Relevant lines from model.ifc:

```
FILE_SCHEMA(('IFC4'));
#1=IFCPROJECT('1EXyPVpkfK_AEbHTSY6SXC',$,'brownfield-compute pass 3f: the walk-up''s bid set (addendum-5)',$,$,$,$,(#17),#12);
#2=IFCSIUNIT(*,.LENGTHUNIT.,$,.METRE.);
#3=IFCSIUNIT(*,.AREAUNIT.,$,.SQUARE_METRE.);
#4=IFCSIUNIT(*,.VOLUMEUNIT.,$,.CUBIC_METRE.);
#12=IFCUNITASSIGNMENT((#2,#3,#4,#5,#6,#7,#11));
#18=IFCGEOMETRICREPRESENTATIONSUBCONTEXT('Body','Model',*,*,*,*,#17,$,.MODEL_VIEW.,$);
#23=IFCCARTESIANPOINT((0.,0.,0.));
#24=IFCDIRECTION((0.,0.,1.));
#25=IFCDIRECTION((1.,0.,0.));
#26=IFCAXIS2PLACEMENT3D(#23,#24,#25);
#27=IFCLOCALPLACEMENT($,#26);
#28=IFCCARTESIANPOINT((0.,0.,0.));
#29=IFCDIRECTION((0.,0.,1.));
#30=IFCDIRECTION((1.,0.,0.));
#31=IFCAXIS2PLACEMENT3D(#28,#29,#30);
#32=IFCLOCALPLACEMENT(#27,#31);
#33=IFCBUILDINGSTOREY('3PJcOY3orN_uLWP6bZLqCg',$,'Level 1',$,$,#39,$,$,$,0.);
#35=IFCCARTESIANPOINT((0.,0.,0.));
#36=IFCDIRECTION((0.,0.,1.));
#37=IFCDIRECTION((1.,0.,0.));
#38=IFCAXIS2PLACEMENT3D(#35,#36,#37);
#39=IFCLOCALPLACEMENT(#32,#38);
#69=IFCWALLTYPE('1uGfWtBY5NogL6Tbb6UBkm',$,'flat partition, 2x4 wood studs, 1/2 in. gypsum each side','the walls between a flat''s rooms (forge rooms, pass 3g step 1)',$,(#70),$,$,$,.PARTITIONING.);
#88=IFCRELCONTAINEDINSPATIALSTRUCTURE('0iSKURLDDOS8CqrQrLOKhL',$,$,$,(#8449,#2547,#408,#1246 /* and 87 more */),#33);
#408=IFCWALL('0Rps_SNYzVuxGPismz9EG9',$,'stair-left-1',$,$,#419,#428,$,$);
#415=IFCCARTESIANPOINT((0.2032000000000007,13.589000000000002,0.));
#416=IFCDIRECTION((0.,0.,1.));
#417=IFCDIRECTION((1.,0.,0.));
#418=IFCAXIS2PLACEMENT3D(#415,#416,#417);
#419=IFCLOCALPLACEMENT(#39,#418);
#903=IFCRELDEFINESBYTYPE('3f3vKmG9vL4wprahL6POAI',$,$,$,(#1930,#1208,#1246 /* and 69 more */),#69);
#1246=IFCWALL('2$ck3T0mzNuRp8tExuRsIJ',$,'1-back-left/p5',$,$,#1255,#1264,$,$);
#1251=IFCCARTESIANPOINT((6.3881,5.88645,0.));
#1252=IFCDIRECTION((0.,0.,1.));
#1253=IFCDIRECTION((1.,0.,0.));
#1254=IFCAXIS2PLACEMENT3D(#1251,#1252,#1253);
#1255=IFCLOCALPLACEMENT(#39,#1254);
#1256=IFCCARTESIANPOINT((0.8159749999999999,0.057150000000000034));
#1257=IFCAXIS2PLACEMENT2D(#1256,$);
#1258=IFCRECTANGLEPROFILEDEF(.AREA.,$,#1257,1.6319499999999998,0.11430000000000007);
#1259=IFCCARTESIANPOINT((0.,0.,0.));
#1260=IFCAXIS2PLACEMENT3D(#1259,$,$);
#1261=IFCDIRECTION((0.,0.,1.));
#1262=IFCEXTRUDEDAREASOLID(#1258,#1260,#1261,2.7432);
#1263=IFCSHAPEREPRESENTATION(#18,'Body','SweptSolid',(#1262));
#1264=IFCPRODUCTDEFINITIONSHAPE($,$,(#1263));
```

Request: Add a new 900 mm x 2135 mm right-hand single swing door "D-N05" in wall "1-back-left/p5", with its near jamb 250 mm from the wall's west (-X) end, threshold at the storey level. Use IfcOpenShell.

```python
import numpy as np
import ifcopenshell
import ifcopenshell.api.feature
import ifcopenshell.api.geometry
import ifcopenshell.api.root
import ifcopenshell.api.spatial
import ifcopenshell.geom
import ifcopenshell.util.element
import ifcopenshell.util.placement
import ifcopenshell.util.representation
import ifcopenshell.util.shape
import ifcopenshell.util.unit

model = ifcopenshell.open("model.ifc")
unit_scale = ifcopenshell.util.unit.calculate_unit_scale(model)
settings = ifcopenshell.geom.settings()


def volume(element):
    """Net volume in cubic metres, openings subtracted."""
    shape = ifcopenshell.geom.create_shape(settings, element)
    return ifcopenshell.util.shape.get_volume(shape.geometry)


wall = model.by_guid("2$ck3T0mzNuRp8tExuRsIJ")
storey = ifcopenshell.util.element.get_container(wall, ifc_class="IfcBuildingStorey")
context = ifcopenshell.util.representation.get_context(model, "Model", "Body", "MODEL_VIEW")
before = volume(wall)

width, height, from_end, sill = 0.9, 2.135, 0.25, 0.0  # metres

# The wall runs along its own X axis, and the end named is its -X end.
wall_shape = ifcopenshell.geom.create_shape(settings, wall)
x, y, z = ifcopenshell.util.shape.get_vertices(wall_shape.geometry).T
start = x.min() + from_end
face, thickness = float(y.min()), float(y.max() - y.min())
wall_matrix = ifcopenshell.util.placement.get_local_placement(wall.ObjectPlacement)
level = ifcopenshell.util.placement.get_local_placement(storey.ObjectPlacement)[2, 3]


def in_wall(x, y):
    """Placement at x, y metres in the wall's axes, at sill height."""
    matrix = wall_matrix.copy()
    matrix[:, 3] = wall_matrix @ np.array([x / unit_scale, y / unit_scale, 0.0, 1.0])
    matrix[2, 3] = level + sill / unit_scale
    return matrix


# Opening: a box that overshoots both wall faces by 50 mm.
opening = ifcopenshell.api.root.create_entity(model, ifc_class="IfcOpeningElement", predefined_type="OPENING")
box = ifcopenshell.api.geometry.add_wall_representation(
    model, context=context, length=width, height=height, thickness=thickness + 0.1
)
ifcopenshell.api.geometry.assign_representation(model, product=opening, representation=box)
ifcopenshell.api.geometry.edit_object_placement(model, product=opening, matrix=in_wall(start, face - 0.05), is_si=False)
ifcopenshell.api.feature.add_feature(model, feature=opening, element=wall)

door = ifcopenshell.api.root.create_entity(model, ifc_class="IfcDoor", name="D-N05", predefined_type="DOOR")
door.OverallWidth, door.OverallHeight = width / unit_scale, height / unit_scale
door.OperationType = "SINGLE_SWING_RIGHT"
body = ifcopenshell.api.geometry.add_door_representation(
    model,
    context=context,
    overall_width=door.OverallWidth,
    overall_height=door.OverallHeight,
    operation_type="SINGLE_SWING_RIGHT",
    lining_properties={"LiningDepth": thickness / unit_scale, "ThresholdDepth": thickness / unit_scale},
)
ifcopenshell.api.geometry.assign_representation(model, product=door, representation=body)
ifcopenshell.api.spatial.assign_container(model, products=[door], relating_structure=storey)
ifcopenshell.api.feature.add_filling(model, opening=opening, element=door)

# The lining spans the wall, so the door starts at the wall face.
ifcopenshell.api.geometry.edit_object_placement(model, product=door, matrix=in_wall(start, face), is_si=False)

after = volume(wall)

print(f"wall volume {before:.3f} -> {after:.3f} m3")

model.write("model_v2.ifc")
```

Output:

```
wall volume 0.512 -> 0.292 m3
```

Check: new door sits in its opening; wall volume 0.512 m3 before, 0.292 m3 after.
